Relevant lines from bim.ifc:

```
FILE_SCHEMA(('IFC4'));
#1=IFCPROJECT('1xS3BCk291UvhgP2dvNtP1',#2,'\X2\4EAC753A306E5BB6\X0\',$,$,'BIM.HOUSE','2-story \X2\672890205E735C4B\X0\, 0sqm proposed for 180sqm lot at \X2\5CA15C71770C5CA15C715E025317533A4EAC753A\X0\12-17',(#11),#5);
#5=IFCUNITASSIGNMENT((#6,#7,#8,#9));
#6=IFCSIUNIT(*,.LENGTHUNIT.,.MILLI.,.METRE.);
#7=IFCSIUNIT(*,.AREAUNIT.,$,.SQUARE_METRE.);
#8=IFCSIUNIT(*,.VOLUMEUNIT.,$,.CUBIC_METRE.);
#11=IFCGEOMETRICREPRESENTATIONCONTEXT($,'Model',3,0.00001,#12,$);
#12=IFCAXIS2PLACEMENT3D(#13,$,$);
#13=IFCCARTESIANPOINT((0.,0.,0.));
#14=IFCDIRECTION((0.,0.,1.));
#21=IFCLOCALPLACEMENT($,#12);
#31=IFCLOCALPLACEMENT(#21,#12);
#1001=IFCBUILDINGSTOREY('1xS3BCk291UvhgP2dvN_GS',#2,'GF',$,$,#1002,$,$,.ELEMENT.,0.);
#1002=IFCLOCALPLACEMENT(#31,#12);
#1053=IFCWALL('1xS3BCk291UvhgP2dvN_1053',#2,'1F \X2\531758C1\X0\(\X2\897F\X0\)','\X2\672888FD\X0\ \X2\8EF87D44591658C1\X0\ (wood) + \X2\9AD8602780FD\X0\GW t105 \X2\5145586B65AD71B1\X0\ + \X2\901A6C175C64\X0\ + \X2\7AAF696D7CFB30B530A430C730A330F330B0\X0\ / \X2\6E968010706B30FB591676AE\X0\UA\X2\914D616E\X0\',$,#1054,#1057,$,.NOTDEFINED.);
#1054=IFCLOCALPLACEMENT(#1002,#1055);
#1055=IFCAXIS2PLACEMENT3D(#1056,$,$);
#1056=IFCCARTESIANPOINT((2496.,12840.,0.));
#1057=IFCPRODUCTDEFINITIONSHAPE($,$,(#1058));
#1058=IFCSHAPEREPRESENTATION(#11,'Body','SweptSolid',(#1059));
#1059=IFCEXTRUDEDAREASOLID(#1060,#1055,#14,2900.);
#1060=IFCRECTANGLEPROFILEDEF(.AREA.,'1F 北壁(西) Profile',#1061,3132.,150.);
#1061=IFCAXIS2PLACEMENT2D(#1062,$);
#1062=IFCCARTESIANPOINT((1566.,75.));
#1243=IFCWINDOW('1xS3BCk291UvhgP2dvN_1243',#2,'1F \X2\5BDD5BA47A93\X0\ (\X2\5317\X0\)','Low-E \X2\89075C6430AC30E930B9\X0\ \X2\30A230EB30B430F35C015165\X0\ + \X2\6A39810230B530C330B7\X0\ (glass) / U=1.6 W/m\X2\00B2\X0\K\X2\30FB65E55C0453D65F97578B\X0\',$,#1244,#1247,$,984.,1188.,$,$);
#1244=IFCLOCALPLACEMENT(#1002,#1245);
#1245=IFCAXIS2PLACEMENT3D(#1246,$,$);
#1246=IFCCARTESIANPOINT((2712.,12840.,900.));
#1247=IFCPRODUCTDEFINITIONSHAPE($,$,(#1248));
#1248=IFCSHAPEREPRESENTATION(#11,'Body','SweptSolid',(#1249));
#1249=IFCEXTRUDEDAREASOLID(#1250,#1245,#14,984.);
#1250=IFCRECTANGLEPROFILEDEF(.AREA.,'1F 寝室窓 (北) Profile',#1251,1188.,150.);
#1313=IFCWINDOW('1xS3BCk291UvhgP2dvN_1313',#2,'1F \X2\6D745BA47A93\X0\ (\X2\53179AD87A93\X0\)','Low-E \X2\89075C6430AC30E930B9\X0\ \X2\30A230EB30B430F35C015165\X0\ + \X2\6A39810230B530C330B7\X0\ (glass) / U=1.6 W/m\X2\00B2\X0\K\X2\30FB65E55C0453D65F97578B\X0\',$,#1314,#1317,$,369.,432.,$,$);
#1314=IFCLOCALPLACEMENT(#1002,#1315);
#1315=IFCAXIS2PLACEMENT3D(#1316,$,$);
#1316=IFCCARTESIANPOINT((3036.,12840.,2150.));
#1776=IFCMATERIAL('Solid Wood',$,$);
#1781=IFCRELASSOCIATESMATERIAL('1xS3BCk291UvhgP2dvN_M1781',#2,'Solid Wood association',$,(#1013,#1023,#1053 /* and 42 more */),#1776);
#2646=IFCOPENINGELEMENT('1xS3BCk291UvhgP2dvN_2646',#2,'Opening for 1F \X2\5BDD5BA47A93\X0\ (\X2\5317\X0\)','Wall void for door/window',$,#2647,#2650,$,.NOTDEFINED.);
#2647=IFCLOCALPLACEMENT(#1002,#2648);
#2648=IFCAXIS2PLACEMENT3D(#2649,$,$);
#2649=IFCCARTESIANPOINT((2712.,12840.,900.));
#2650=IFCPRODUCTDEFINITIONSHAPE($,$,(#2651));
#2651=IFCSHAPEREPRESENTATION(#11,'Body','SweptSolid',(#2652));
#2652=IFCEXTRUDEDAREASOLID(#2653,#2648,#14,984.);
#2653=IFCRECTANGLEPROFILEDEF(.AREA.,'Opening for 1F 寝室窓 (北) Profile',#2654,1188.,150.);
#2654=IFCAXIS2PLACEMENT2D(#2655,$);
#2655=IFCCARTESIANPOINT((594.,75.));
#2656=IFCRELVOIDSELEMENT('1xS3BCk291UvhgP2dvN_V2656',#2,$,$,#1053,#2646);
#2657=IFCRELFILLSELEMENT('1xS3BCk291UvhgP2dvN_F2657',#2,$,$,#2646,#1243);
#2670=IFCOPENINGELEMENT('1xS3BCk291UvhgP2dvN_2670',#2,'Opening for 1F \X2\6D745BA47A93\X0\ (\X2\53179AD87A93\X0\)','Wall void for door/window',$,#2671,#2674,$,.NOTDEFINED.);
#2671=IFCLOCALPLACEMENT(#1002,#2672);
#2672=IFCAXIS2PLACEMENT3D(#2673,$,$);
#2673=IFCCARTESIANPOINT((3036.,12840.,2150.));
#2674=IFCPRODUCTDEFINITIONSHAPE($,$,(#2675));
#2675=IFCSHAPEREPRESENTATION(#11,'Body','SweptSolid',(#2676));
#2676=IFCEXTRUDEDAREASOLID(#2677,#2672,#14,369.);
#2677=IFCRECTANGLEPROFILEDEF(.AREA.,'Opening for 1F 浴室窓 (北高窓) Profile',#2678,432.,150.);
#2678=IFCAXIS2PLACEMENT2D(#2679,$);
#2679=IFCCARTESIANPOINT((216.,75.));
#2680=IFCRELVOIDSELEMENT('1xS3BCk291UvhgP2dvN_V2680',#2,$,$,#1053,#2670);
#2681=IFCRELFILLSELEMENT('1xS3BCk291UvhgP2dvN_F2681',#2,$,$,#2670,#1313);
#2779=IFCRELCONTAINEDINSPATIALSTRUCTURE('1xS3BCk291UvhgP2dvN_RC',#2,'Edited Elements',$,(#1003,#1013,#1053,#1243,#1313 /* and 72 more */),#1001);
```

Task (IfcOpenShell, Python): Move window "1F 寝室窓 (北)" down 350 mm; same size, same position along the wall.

```python
import numpy as np
import ifcopenshell
import ifcopenshell.api.geometry
import ifcopenshell.util.placement
import ifcopenshell.util.unit

model = ifcopenshell.open("bim.ifc")
unit_scale = ifcopenshell.util.unit.calculate_unit_scale(model)

window = model.by_guid("1xS3BCk291UvhgP2dvN_1243")
opening = window.FillsVoids[0].RelatingOpeningElement
dz = -350.0

shift = np.array([0.0, 0.0, dz])
# The window is not placed relative to its opening, so move both.
for product in (opening, window):
    matrix = ifcopenshell.util.placement.get_local_placement(product.ObjectPlacement)
    matrix[:3, 3] += shift
    ifcopenshell.api.geometry.edit_object_placement(model, product=product, matrix=matrix, is_si=False)

print(f"moved by {dz * unit_scale:+.3f} m")

model.write("bim_edited.ifc")
```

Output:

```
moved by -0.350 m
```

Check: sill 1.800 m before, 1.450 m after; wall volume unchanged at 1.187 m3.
